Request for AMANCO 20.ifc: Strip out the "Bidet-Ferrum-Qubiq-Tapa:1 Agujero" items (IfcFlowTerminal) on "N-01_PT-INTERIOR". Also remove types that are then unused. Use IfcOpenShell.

First a look at what the model holds.

```python
import ifcopenshell
import ifcopenshell.util.element

model = ifcopenshell.open("AMANCO 20.ifc")
print(model.schema)
storey = next(s for s in model.by_type("IfcBuildingStorey") if s.Name == "N-01_PT-INTERIOR")
terminals = [e for e in ifcopenshell.util.element.get_decomposition(storey) if e.is_a("IfcFlowTerminal")]
seen = {}
for e in terminals:
    element_type = ifcopenshell.util.element.get_type(e)
    name = element_type.Name if element_type not in (None, e) else None
    seen[name] = seen.get(name, 0) + 1
for name, count in sorted(seen.items(), key=str):
    print(count, "x", name)
```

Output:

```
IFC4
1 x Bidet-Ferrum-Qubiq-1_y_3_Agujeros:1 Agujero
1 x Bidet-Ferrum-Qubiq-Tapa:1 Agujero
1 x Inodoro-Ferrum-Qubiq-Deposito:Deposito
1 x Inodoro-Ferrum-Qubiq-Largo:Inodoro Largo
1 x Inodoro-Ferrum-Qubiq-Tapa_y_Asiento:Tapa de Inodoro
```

```python
import ifcopenshell
import ifcopenshell.api.root
import ifcopenshell.util.element

model = ifcopenshell.open("AMANCO 20.ifc")

storey = next(s for s in model.by_type("IfcBuildingStorey") if s.Name == "N-01_PT-INTERIOR")
terminals = [e for e in ifcopenshell.util.element.get_decomposition(storey) if e.is_a("IfcFlowTerminal")]
targets = [e for e in terminals if (t := ifcopenshell.util.element.get_type(e)) not in (None, e) and t.Name == "Bidet-Ferrum-Qubiq-Tapa:1 Agujero"]
types = {ifcopenshell.util.element.get_type(e) for e in targets} - {None, *targets}

for e in targets:
    ifcopenshell.api.root.remove_product(model, product=e)
print(len(targets), "removed")

unused = [t for t in types if not ifcopenshell.util.element.get_types(t)]
for t in unused:
    ifcopenshell.api.root.remove_product(model, product=t)
print(len(unused), "unused types removed")

model.write("AMANCO 20-out.ifc")
```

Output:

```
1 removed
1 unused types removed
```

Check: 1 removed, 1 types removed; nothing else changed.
